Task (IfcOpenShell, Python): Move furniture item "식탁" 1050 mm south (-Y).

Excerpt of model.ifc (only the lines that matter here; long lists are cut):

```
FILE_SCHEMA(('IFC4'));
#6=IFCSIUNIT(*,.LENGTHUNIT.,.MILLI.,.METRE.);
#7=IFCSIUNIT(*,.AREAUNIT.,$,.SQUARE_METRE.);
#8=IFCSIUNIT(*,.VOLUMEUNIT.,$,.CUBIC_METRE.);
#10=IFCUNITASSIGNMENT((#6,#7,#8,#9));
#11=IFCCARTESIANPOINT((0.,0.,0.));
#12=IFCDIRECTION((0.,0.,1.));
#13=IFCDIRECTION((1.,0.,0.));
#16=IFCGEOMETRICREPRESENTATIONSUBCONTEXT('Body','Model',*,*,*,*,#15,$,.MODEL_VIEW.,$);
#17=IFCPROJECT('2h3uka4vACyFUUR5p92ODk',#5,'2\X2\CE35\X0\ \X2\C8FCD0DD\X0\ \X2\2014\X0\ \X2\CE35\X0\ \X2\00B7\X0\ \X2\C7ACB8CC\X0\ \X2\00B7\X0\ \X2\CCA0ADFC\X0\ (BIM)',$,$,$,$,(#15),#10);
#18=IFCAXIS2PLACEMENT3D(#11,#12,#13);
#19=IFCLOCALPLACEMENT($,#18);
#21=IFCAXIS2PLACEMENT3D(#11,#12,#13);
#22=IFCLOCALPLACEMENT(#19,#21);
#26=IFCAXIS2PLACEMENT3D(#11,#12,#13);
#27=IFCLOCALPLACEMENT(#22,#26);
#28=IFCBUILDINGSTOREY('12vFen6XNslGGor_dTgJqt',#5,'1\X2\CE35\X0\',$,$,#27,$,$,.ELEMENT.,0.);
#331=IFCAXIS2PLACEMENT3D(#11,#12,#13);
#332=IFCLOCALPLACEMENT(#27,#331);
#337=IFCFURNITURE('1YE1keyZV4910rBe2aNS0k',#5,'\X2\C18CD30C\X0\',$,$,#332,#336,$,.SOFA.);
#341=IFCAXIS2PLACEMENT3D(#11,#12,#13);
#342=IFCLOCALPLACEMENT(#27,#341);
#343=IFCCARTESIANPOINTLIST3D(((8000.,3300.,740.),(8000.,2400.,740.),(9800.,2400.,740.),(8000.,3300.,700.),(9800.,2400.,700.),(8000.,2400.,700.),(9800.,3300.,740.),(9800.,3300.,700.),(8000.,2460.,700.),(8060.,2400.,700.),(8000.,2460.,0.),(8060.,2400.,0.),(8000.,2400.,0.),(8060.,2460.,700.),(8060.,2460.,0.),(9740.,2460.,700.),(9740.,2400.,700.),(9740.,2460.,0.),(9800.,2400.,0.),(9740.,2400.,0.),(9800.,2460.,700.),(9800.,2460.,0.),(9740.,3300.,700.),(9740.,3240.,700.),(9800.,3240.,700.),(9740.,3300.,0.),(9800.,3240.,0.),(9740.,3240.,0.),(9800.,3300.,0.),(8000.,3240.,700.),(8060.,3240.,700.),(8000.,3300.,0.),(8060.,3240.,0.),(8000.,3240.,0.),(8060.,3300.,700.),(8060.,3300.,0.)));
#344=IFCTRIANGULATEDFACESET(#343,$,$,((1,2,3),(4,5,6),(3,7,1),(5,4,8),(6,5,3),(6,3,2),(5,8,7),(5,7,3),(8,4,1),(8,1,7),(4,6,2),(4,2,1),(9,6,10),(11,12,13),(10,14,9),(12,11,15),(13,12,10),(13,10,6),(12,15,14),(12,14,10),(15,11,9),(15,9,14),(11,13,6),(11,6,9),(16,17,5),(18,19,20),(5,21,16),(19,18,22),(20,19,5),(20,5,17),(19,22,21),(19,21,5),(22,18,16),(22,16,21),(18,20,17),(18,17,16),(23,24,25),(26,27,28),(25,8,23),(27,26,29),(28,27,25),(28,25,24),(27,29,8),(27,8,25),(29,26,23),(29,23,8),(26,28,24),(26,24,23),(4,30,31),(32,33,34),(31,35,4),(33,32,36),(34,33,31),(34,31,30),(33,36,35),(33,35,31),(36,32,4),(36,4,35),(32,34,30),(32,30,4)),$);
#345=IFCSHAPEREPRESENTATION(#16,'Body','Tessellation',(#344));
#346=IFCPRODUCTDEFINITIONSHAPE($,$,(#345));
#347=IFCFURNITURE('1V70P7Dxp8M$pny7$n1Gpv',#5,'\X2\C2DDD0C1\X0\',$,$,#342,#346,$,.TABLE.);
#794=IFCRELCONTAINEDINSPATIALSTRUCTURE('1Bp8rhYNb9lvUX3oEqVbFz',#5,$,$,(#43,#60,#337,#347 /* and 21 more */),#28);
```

```python
import ifcopenshell
import ifcopenshell.api.geometry
import ifcopenshell.util.placement

model = ifcopenshell.open("model.ifc")

item = model.by_guid("1V70P7Dxp8M$pny7$n1Gpv")
matrix = ifcopenshell.util.placement.get_local_placement(item.ObjectPlacement)
matrix[1, 3] -= 1050.0
ifcopenshell.api.geometry.edit_object_placement(model, product=item, matrix=matrix, is_si=False)

print(ifcopenshell.util.placement.get_local_placement(item.ObjectPlacement).round(3) + 0.0)

model.write("model_edited.ifc")
```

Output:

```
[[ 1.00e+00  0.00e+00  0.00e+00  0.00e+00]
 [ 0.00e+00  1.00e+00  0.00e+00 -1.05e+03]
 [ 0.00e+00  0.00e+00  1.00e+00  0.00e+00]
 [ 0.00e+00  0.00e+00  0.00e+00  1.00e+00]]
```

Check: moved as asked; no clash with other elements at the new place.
